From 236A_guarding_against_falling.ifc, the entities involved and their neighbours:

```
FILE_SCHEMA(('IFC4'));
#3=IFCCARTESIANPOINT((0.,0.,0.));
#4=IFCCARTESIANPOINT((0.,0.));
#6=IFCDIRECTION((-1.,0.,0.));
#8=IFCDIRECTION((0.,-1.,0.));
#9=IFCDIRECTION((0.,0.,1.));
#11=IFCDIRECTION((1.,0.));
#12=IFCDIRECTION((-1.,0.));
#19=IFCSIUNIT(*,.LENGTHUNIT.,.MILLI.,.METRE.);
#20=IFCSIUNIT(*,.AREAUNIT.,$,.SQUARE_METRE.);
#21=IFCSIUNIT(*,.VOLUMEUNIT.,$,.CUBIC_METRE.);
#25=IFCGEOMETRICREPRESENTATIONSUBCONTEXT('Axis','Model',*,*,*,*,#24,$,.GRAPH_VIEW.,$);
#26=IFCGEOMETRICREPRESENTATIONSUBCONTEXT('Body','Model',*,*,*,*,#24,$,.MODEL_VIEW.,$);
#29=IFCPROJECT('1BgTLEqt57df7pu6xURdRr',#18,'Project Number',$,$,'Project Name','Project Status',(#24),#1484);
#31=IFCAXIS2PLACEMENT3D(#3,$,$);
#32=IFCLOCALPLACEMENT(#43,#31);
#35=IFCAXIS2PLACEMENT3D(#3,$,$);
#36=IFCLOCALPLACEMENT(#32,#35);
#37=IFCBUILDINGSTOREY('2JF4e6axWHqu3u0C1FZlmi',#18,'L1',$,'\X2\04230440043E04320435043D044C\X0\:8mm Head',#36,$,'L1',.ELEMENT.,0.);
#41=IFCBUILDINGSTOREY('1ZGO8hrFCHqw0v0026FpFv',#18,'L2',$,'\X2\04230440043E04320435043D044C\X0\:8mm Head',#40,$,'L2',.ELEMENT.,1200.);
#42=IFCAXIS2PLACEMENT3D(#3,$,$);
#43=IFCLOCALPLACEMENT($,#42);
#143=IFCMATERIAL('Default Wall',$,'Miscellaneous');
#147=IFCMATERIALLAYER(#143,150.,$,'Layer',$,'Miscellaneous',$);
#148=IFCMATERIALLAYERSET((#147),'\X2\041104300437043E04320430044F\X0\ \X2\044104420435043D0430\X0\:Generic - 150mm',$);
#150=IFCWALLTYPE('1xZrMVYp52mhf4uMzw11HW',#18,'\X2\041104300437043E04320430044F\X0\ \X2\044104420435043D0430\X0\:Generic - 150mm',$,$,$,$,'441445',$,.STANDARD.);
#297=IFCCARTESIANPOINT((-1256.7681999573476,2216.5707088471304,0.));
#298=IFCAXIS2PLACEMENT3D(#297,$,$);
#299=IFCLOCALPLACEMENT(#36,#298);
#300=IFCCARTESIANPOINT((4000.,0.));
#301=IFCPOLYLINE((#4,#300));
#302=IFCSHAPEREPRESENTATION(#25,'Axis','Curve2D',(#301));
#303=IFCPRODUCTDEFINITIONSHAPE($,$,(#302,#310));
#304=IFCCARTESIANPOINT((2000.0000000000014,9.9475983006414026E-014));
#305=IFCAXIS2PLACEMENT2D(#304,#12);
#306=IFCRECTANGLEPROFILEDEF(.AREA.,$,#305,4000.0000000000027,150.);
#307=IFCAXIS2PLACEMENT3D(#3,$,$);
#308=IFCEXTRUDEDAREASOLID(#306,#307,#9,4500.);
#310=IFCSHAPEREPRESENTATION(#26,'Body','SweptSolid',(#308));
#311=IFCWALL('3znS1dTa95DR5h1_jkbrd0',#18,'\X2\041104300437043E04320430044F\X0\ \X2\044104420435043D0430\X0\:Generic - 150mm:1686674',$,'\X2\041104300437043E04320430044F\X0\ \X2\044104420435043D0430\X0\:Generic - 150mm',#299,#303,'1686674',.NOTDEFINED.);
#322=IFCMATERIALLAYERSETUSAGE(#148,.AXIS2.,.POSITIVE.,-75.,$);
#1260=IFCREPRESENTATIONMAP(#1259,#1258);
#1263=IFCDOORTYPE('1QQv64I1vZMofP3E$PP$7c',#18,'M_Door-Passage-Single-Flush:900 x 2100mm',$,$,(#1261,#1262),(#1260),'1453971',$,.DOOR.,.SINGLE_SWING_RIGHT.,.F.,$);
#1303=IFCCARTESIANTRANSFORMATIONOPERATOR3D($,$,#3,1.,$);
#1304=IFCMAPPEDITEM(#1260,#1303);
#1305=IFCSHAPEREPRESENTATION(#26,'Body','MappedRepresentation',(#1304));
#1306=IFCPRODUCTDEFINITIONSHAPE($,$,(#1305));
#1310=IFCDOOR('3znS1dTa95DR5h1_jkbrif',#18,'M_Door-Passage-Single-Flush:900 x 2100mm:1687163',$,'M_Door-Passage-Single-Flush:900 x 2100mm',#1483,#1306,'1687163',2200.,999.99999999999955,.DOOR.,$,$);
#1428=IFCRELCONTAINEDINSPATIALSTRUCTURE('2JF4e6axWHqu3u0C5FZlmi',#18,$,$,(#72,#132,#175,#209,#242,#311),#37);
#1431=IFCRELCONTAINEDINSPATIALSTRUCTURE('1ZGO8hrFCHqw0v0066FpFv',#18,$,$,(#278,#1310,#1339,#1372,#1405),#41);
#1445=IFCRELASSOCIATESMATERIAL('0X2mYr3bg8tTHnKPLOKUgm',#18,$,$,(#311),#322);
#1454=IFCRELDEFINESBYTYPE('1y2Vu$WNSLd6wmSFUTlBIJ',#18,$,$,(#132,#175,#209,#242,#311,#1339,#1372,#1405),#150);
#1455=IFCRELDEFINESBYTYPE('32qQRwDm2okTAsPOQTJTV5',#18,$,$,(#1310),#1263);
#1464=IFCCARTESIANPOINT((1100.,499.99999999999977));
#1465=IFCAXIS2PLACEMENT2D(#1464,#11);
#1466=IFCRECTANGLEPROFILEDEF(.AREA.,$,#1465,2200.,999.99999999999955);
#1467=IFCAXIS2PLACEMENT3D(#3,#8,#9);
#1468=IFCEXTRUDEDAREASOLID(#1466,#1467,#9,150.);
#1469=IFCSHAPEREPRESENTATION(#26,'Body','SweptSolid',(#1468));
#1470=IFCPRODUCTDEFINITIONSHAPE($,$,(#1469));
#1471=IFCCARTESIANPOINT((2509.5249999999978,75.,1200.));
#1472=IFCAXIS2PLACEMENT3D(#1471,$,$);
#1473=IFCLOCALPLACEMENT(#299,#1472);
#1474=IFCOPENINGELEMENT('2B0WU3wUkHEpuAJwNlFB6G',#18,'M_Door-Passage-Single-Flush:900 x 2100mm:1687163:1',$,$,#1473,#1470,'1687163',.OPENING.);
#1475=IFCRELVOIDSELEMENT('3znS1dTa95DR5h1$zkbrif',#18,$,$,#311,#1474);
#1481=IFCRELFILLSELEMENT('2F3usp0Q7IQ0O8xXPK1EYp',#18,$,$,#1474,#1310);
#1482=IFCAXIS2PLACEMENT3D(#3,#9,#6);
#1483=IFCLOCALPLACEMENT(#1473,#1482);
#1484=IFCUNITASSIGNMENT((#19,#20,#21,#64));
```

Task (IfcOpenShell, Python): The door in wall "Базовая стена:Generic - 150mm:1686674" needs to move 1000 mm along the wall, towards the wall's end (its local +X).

```python
import ifcopenshell
import ifcopenshell.api.geometry
import ifcopenshell.util.placement
import ifcopenshell.util.unit

model = ifcopenshell.open("236A_guarding_against_falling.ifc")
unit_scale = ifcopenshell.util.unit.calculate_unit_scale(model)

door = model.by_guid("3znS1dTa95DR5h1_jkbrif")
opening = door.FillsVoids[0].RelatingOpeningElement
wall = opening.VoidsElements[0].RelatingBuildingElement

wall_matrix = ifcopenshell.util.placement.get_local_placement(wall.ObjectPlacement)
shift = wall_matrix[:3, 0] * 1 / unit_scale
before = ifcopenshell.util.placement.get_local_placement(door.ObjectPlacement)[:3, 3].copy()

# The door is placed relative to its opening, so it follows when the opening moves.
matrix = ifcopenshell.util.placement.get_local_placement(opening.ObjectPlacement)
matrix[:3, 3] += shift
ifcopenshell.api.geometry.edit_object_placement(
    model, product=opening, matrix=matrix, is_si=False, should_transform_children=True
)

after = ifcopenshell.util.placement.get_local_placement(door.ObjectPlacement)[:3, 3]
print("door moved by", (after - before).round(3) + 0.0)

model.write("236A_guarding_against_falling_rev.ifc")
```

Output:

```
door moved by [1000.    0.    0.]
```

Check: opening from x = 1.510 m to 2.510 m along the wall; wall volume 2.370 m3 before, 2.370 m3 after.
